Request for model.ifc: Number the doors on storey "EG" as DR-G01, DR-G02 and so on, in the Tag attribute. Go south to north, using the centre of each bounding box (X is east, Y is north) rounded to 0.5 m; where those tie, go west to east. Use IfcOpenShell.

First a look at what the model holds.

```python
import ifcopenshell
import ifcopenshell.util.element
import ifcopenshell.util.placement

model = ifcopenshell.open("model.ifc")
print(model.schema)
storey = next(s for s in model.by_type("IfcBuildingStorey") if s.Name == "EG")
doors = [e for e in ifcopenshell.util.element.get_decomposition(storey) if e.is_a("IfcDoor")]
for e in sorted(doors, key=lambda e: e.id()):
    origin = ifcopenshell.util.placement.get_local_placement(e.ObjectPlacement)[:3, 3]
    print(e.id(), e.Tag, e.Name, origin.round(2) + 0.0, sep=" | ")
```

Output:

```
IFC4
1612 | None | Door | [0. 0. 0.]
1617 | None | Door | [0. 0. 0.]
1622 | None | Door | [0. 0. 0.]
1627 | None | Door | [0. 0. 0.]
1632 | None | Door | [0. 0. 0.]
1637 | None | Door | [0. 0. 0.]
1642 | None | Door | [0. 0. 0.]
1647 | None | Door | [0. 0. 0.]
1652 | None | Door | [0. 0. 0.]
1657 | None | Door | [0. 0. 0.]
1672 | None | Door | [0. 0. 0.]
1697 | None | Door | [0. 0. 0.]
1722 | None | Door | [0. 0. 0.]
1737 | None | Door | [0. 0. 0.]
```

```python
import ifcopenshell
import ifcopenshell.geom
import ifcopenshell.util.element
import ifcopenshell.util.shape

model = ifcopenshell.open("model.ifc")
settings = ifcopenshell.geom.settings()
settings.set("use-world-coords", True)


def centre(element):
    shape = ifcopenshell.geom.create_shape(settings, element)
    return ifcopenshell.util.shape.get_bbox_centroid(shape.geometry)


storey = next(s for s in model.by_type("IfcBuildingStorey") if s.Name == "EG")
doors = [e for e in ifcopenshell.util.element.get_decomposition(storey) if e.is_a("IfcDoor")]

# Insertion points can sit at a corner or the storey origin, so sort by the geometry (in metres).
centres = {e: centre(e) for e in doors}
doors.sort(key=lambda e: (round(centres[e][1] / 0.5), centres[e][0]))

for i, e in enumerate(doors, start=1):
    number = f"DR-G{i:02d}"
    e.Tag = number
    print(e.id(), number)

model.write("model_edited.ifc")
```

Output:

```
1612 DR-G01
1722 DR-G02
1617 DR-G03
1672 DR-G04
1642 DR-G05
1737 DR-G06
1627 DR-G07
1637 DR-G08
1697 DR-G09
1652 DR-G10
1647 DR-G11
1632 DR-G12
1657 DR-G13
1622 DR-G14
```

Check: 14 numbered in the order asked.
